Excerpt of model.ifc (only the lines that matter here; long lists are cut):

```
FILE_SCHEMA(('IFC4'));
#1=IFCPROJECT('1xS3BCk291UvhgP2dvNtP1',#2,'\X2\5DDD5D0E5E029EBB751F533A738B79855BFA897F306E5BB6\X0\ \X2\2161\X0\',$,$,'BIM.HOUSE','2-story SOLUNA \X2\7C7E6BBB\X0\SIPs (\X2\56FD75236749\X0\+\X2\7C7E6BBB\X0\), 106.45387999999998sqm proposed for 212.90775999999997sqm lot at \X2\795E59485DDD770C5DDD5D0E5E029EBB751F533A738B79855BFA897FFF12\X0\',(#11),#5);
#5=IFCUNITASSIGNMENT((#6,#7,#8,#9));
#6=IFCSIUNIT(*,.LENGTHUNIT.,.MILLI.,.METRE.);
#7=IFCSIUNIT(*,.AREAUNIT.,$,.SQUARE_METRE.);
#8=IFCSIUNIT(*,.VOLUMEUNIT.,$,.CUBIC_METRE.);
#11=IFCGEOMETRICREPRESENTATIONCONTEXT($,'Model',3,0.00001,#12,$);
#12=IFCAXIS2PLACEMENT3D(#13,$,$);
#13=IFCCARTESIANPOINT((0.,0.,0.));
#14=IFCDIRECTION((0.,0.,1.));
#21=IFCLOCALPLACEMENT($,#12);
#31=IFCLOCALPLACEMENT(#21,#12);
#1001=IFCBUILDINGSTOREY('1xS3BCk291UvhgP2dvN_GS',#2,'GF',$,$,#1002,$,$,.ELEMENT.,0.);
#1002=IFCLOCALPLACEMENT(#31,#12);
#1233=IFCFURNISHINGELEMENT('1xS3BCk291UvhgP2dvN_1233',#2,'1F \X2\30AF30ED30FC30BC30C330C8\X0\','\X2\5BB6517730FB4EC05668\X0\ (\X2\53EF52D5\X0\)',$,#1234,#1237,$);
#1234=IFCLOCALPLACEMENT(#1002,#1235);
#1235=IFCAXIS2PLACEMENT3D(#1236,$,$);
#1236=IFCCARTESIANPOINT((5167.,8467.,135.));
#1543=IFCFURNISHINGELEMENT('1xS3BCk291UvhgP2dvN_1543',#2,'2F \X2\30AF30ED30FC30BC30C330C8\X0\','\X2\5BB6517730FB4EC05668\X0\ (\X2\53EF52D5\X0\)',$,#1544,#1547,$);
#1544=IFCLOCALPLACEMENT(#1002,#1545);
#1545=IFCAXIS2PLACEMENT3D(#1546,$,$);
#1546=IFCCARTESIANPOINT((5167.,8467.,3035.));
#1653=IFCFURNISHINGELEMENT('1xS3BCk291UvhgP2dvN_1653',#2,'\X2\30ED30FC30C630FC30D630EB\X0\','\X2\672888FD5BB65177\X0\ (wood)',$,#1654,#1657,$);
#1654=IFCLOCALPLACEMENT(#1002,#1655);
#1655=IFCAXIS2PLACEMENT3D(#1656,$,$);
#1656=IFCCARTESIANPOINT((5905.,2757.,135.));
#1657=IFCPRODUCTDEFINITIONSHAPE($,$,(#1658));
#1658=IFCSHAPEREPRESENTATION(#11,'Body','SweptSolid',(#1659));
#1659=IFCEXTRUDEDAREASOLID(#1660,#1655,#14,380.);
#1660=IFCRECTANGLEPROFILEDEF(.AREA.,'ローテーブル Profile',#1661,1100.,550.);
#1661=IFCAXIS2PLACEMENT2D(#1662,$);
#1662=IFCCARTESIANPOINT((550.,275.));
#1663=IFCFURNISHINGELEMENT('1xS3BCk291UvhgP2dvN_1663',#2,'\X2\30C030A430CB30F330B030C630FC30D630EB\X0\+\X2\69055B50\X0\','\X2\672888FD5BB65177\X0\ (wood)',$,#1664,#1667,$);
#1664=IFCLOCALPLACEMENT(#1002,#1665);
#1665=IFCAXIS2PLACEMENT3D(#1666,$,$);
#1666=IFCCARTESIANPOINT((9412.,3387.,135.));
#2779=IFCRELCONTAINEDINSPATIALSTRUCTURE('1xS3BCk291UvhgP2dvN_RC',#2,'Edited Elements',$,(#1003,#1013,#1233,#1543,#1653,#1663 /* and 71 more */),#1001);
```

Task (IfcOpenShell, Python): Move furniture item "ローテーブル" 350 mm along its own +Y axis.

```python
import ifcopenshell
import ifcopenshell.api.geometry
import ifcopenshell.util.placement

model = ifcopenshell.open("model.ifc")

item = model.by_id(1653)
matrix = ifcopenshell.util.placement.get_local_placement(item.ObjectPlacement)
matrix[:3, 3] += matrix[:3, 1] * 350.0
ifcopenshell.api.geometry.edit_object_placement(model, product=item, matrix=matrix, is_si=False)

print(ifcopenshell.util.placement.get_local_placement(item.ObjectPlacement).round(3) + 0.0)

model.write("model_rev.ifc")
```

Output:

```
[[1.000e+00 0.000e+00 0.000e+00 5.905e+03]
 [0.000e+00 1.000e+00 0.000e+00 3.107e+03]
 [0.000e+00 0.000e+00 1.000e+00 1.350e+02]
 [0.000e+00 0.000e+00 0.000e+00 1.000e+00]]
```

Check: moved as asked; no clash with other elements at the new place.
